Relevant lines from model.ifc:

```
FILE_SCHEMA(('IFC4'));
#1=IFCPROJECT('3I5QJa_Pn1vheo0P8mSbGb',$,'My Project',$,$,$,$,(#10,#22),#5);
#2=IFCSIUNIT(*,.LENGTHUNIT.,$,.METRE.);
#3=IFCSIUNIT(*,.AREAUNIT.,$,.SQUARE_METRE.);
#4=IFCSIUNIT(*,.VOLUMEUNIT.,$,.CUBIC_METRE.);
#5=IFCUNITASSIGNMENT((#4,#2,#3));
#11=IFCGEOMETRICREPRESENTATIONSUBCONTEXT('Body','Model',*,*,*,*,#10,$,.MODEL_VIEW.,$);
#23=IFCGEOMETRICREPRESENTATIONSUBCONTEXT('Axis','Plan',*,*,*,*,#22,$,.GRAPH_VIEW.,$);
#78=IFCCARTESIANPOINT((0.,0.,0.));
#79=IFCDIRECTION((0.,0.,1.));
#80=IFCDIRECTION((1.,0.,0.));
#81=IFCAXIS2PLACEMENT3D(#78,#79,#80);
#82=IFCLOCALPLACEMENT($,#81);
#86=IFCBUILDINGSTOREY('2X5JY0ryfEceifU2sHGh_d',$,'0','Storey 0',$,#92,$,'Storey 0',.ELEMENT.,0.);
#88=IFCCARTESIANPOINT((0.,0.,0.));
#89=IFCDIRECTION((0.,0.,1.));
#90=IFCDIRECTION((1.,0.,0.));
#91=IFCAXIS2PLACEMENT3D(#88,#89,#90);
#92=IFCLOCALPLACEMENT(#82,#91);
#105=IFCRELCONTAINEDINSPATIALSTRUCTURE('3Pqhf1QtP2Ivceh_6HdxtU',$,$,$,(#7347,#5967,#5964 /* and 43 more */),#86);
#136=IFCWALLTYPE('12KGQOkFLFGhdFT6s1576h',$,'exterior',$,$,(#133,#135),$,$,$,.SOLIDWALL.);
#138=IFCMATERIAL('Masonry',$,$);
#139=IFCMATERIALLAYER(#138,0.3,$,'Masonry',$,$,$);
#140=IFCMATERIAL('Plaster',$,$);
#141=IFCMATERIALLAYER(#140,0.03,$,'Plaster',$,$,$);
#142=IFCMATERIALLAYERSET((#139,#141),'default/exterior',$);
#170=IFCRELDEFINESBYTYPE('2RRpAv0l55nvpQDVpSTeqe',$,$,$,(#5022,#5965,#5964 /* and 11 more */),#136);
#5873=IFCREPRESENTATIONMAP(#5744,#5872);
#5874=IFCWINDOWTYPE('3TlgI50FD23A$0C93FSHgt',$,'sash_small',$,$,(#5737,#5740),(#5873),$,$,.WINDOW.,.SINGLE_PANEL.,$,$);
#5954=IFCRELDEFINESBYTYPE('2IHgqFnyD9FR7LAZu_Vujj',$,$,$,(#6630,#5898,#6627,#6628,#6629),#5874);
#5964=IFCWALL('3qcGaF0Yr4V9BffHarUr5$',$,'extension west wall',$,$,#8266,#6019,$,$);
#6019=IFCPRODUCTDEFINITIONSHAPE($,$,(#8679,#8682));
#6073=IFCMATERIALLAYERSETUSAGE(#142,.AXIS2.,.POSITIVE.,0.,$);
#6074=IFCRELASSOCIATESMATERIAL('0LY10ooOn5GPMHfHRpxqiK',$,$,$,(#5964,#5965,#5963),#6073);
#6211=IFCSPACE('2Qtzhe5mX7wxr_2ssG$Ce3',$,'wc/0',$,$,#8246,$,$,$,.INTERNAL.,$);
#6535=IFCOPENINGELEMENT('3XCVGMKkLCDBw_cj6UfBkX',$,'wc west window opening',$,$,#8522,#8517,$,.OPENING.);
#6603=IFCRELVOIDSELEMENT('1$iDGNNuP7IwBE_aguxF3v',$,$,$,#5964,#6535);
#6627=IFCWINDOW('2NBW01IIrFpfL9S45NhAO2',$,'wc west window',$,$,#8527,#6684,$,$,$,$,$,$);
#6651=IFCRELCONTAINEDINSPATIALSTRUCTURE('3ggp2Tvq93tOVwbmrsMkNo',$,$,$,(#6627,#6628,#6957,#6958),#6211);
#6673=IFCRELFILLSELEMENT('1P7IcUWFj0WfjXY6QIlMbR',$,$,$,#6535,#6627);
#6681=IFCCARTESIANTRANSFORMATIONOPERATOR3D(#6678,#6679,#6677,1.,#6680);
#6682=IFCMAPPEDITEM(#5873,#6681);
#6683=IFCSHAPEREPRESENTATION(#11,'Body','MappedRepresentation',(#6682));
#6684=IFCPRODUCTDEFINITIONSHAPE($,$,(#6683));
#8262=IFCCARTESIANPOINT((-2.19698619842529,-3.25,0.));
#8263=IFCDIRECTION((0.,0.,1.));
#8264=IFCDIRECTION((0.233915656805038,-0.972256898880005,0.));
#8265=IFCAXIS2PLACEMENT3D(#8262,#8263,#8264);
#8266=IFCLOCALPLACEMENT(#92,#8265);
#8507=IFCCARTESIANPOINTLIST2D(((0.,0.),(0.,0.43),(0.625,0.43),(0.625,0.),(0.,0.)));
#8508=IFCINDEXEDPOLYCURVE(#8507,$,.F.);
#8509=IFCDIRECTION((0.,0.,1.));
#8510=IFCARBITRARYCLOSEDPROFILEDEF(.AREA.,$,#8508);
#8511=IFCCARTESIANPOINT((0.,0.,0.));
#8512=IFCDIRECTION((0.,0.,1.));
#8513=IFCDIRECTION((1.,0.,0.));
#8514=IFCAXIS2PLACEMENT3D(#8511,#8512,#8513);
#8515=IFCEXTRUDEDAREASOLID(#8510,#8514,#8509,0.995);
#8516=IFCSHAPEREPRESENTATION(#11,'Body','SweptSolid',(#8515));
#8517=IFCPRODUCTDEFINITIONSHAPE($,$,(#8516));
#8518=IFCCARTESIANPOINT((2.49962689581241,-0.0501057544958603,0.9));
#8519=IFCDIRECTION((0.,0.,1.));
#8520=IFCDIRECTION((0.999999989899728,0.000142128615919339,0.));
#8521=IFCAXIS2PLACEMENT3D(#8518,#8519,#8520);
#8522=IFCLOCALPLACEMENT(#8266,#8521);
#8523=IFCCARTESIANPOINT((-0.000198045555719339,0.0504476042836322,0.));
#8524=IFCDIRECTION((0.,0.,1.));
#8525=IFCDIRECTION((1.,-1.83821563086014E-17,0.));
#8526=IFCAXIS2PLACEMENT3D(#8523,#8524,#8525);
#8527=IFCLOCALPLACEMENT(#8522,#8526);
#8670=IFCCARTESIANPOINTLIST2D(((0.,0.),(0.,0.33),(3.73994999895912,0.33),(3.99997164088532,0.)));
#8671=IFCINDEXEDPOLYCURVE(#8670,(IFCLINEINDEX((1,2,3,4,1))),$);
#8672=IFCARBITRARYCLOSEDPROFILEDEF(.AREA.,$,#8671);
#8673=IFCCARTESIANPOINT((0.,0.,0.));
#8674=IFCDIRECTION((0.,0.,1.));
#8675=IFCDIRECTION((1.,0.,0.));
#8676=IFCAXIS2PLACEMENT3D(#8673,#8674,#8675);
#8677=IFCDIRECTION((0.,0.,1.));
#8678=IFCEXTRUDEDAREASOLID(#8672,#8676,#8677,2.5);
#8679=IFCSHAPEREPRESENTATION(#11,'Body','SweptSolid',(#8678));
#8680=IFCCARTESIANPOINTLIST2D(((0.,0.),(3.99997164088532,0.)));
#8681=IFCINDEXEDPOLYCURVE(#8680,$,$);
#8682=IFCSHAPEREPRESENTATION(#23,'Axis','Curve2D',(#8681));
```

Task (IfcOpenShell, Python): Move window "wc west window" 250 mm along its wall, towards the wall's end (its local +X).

```python
import ifcopenshell
import ifcopenshell.api.geometry
import ifcopenshell.util.placement
import ifcopenshell.util.unit

model = ifcopenshell.open("model.ifc")
unit_scale = ifcopenshell.util.unit.calculate_unit_scale(model)

window = model.by_guid("2NBW01IIrFpfL9S45NhAO2")
opening = window.FillsVoids[0].RelatingOpeningElement
wall = opening.VoidsElements[0].RelatingBuildingElement

wall_matrix = ifcopenshell.util.placement.get_local_placement(wall.ObjectPlacement)
shift = wall_matrix[:3, 0] * 0.25 / unit_scale
before = ifcopenshell.util.placement.get_local_placement(window.ObjectPlacement)[:3, 3].copy()

# The window is placed relative to its opening, so it follows when the opening moves.
matrix = ifcopenshell.util.placement.get_local_placement(opening.ObjectPlacement)
matrix[:3, 3] += shift
ifcopenshell.api.geometry.edit_object_placement(
    model, product=opening, matrix=matrix, is_si=False, should_transform_children=True
)

after = ifcopenshell.util.placement.get_local_placement(window.ObjectPlacement)[:3, 3]
print("window moved by", (after - before).round(3) + 0.0)

model.write("model-out.ifc")
```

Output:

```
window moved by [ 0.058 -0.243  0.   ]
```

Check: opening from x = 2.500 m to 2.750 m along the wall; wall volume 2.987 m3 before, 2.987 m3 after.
